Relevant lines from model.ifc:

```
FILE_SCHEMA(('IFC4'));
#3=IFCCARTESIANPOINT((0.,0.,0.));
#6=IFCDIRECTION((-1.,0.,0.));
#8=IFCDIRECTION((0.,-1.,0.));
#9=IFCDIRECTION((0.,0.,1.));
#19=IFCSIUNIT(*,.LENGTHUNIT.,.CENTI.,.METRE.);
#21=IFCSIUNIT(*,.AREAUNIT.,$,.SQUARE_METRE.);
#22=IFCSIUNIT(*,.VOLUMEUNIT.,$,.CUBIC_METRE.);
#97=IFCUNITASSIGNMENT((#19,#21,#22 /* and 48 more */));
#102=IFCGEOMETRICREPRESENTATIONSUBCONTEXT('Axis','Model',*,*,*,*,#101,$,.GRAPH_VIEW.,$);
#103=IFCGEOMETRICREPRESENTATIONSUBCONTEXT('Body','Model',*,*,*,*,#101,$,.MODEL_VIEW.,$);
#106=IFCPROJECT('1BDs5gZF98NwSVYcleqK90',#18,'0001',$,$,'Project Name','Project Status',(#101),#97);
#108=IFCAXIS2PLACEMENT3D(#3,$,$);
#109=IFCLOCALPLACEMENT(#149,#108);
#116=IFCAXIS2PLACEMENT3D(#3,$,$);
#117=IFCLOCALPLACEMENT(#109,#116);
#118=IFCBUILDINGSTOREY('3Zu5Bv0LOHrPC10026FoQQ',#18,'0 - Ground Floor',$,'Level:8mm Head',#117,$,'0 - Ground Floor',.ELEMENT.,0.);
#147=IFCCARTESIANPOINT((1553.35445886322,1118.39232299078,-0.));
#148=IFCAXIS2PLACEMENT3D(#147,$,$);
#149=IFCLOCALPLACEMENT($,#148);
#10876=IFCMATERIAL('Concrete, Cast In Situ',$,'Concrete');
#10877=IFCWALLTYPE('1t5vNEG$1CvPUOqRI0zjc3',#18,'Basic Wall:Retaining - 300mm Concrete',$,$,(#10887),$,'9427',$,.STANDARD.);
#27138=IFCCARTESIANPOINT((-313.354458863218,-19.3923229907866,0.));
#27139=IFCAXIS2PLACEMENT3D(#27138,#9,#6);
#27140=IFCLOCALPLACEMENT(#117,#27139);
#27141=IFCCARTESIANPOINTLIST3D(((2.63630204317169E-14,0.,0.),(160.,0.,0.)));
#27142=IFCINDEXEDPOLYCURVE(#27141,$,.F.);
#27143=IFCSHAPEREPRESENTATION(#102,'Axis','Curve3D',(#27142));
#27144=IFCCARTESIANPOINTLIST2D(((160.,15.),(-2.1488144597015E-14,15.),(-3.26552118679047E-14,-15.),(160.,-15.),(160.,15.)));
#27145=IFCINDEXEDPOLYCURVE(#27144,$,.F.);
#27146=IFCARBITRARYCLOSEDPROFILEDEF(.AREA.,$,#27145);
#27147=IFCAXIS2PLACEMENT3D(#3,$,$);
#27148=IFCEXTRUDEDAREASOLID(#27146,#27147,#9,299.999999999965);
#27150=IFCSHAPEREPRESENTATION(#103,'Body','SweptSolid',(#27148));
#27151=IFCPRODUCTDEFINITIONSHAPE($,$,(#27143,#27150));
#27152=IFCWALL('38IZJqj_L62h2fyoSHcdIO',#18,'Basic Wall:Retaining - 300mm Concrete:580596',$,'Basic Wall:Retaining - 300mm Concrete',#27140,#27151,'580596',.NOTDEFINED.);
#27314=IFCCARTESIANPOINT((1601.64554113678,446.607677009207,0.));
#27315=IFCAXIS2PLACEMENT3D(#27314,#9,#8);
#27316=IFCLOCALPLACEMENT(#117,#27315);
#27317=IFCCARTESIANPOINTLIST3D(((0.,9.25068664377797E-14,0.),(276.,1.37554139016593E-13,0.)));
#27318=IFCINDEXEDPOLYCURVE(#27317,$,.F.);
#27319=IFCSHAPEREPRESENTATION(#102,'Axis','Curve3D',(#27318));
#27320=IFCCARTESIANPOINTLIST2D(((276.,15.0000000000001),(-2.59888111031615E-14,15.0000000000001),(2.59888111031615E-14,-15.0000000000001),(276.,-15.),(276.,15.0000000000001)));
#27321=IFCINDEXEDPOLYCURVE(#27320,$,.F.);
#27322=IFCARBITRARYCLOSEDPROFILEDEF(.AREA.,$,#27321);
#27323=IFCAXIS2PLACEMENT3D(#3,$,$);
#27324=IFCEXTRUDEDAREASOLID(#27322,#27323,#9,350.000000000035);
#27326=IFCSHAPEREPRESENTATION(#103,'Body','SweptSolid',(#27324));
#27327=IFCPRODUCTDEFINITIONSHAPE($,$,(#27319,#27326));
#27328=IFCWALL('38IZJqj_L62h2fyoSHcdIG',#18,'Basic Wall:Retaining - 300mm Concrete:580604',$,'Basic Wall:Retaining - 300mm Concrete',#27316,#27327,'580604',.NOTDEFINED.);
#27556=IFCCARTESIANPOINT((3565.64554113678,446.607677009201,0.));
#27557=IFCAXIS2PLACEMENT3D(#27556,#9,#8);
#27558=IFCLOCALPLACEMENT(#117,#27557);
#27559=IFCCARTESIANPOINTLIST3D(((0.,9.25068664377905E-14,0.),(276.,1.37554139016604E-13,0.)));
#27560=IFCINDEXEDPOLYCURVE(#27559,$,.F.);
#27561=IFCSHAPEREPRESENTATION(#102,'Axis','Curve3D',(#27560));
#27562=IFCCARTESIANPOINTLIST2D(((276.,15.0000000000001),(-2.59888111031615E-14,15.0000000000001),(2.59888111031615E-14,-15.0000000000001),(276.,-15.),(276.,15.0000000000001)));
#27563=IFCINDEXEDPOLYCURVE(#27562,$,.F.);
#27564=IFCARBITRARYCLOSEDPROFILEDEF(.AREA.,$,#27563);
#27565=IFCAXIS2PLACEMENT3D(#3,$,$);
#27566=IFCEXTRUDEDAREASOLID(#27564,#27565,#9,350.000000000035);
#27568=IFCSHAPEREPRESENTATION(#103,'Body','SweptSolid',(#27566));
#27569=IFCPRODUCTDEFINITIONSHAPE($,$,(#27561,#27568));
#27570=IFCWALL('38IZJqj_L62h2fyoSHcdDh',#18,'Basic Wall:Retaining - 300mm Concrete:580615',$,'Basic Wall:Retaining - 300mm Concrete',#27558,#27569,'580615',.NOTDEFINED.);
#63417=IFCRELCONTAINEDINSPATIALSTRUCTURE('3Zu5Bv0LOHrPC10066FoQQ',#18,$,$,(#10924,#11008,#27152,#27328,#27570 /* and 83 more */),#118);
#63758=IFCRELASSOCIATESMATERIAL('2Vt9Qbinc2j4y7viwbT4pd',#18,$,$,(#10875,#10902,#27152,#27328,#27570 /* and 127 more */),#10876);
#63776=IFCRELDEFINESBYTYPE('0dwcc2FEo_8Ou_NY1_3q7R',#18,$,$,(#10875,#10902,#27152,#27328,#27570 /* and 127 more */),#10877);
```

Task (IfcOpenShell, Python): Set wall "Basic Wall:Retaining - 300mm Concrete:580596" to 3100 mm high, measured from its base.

```python
import ifcopenshell
import ifcopenshell.geom
import ifcopenshell.util.representation
import ifcopenshell.util.shape
import ifcopenshell.util.unit

model = ifcopenshell.open("model.ifc")
unit_scale = ifcopenshell.util.unit.calculate_unit_scale(model)
settings = ifcopenshell.geom.settings()


def volume(element):
    """Net volume in cubic metres, openings subtracted."""
    shape = ifcopenshell.geom.create_shape(settings, element)
    return ifcopenshell.util.shape.get_volume(shape.geometry)


wall = model.by_id(27152)
before = volume(wall)

body = ifcopenshell.util.representation.get_representation(wall, "Model", "Body")
solid = body.Items[0]
old_height = solid.Depth
solid.Depth = 3.1 / unit_scale
after = volume(wall)

print(f"height {old_height:g} -> {solid.Depth:g}, volume {before:.3f} -> {after:.3f} m3")

model.write("model-out.ifc")
```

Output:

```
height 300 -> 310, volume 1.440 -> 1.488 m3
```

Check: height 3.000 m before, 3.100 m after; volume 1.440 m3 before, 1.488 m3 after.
